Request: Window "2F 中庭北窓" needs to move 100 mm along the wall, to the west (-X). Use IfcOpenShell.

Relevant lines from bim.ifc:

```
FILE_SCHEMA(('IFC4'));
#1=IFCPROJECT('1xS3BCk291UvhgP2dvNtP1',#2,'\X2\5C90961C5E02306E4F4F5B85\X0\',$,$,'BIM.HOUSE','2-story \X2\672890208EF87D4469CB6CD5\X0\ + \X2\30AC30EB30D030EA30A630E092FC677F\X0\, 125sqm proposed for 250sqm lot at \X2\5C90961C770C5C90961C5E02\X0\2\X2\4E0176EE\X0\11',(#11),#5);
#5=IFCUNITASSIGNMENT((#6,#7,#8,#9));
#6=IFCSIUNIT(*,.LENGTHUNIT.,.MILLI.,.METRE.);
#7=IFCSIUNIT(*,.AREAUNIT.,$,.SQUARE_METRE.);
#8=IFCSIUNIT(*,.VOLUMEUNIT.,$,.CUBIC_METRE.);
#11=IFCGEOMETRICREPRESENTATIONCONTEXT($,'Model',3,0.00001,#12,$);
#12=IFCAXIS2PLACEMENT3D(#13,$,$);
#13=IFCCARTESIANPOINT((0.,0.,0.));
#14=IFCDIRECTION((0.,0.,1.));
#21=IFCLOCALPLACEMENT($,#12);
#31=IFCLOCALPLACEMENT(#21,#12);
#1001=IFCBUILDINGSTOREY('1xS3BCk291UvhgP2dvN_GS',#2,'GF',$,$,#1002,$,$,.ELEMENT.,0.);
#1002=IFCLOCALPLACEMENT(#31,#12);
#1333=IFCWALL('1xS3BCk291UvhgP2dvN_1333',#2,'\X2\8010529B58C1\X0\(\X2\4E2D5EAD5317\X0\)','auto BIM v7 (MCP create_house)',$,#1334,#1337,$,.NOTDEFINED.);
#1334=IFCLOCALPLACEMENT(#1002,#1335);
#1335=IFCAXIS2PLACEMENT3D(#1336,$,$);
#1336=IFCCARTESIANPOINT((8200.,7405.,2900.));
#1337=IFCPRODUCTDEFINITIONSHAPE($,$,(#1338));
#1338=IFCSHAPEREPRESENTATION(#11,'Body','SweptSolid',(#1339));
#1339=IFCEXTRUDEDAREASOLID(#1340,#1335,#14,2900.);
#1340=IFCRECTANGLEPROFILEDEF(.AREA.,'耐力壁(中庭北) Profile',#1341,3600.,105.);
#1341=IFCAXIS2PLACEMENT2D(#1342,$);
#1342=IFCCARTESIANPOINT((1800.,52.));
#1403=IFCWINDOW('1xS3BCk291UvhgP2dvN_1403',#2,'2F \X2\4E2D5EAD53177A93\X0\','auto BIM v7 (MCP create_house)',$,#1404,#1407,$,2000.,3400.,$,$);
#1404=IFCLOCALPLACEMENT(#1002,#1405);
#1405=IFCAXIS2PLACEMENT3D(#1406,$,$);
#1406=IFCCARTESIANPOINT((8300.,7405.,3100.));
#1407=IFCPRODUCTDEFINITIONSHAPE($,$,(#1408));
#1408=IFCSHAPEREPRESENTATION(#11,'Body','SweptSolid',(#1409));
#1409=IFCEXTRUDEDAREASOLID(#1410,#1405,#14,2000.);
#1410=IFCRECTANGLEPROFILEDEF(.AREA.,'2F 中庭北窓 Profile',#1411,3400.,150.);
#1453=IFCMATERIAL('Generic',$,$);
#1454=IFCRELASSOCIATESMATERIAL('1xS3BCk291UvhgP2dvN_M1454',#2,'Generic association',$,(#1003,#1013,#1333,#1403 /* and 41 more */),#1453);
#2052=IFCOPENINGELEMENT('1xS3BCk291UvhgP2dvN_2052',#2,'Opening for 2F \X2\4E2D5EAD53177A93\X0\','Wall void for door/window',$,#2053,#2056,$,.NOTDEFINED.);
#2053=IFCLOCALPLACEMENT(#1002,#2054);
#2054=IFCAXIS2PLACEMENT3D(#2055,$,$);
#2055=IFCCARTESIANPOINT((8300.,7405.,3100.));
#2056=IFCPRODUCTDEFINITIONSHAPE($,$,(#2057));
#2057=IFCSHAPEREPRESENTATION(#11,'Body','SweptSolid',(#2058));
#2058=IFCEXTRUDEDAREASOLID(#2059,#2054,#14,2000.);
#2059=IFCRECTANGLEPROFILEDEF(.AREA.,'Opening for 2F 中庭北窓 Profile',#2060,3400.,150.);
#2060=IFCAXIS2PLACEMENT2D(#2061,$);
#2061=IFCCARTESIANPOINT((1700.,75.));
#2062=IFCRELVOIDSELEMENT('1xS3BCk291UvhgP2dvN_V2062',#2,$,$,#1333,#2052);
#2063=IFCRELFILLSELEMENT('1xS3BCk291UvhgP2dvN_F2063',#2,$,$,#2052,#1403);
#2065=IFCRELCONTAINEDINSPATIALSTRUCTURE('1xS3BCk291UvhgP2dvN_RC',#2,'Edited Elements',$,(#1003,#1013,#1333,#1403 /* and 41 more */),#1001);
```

```python
import ifcopenshell
import ifcopenshell.api.geometry
import ifcopenshell.util.placement
import ifcopenshell.util.unit

model = ifcopenshell.open("bim.ifc")
unit_scale = ifcopenshell.util.unit.calculate_unit_scale(model)

window = model.by_guid("1xS3BCk291UvhgP2dvN_1403")
opening = window.FillsVoids[0].RelatingOpeningElement
wall = opening.VoidsElements[0].RelatingBuildingElement

wall_matrix = ifcopenshell.util.placement.get_local_placement(wall.ObjectPlacement)
shift = wall_matrix[:3, 0] * -0.1 / unit_scale
before = ifcopenshell.util.placement.get_local_placement(window.ObjectPlacement)[:3, 3].copy()

# The window is not placed relative to its opening, so move both.
for product in (opening, window):
    matrix = ifcopenshell.util.placement.get_local_placement(product.ObjectPlacement)
    matrix[:3, 3] += shift
    ifcopenshell.api.geometry.edit_object_placement(model, product=product, matrix=matrix, is_si=False)

after = ifcopenshell.util.placement.get_local_placement(window.ObjectPlacement)[:3, 3]
print("window moved by", (after - before).round(3) + 0.0)

model.write("bim_updated.ifc")
```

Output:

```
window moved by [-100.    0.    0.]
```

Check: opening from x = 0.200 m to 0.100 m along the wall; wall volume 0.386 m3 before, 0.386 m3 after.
